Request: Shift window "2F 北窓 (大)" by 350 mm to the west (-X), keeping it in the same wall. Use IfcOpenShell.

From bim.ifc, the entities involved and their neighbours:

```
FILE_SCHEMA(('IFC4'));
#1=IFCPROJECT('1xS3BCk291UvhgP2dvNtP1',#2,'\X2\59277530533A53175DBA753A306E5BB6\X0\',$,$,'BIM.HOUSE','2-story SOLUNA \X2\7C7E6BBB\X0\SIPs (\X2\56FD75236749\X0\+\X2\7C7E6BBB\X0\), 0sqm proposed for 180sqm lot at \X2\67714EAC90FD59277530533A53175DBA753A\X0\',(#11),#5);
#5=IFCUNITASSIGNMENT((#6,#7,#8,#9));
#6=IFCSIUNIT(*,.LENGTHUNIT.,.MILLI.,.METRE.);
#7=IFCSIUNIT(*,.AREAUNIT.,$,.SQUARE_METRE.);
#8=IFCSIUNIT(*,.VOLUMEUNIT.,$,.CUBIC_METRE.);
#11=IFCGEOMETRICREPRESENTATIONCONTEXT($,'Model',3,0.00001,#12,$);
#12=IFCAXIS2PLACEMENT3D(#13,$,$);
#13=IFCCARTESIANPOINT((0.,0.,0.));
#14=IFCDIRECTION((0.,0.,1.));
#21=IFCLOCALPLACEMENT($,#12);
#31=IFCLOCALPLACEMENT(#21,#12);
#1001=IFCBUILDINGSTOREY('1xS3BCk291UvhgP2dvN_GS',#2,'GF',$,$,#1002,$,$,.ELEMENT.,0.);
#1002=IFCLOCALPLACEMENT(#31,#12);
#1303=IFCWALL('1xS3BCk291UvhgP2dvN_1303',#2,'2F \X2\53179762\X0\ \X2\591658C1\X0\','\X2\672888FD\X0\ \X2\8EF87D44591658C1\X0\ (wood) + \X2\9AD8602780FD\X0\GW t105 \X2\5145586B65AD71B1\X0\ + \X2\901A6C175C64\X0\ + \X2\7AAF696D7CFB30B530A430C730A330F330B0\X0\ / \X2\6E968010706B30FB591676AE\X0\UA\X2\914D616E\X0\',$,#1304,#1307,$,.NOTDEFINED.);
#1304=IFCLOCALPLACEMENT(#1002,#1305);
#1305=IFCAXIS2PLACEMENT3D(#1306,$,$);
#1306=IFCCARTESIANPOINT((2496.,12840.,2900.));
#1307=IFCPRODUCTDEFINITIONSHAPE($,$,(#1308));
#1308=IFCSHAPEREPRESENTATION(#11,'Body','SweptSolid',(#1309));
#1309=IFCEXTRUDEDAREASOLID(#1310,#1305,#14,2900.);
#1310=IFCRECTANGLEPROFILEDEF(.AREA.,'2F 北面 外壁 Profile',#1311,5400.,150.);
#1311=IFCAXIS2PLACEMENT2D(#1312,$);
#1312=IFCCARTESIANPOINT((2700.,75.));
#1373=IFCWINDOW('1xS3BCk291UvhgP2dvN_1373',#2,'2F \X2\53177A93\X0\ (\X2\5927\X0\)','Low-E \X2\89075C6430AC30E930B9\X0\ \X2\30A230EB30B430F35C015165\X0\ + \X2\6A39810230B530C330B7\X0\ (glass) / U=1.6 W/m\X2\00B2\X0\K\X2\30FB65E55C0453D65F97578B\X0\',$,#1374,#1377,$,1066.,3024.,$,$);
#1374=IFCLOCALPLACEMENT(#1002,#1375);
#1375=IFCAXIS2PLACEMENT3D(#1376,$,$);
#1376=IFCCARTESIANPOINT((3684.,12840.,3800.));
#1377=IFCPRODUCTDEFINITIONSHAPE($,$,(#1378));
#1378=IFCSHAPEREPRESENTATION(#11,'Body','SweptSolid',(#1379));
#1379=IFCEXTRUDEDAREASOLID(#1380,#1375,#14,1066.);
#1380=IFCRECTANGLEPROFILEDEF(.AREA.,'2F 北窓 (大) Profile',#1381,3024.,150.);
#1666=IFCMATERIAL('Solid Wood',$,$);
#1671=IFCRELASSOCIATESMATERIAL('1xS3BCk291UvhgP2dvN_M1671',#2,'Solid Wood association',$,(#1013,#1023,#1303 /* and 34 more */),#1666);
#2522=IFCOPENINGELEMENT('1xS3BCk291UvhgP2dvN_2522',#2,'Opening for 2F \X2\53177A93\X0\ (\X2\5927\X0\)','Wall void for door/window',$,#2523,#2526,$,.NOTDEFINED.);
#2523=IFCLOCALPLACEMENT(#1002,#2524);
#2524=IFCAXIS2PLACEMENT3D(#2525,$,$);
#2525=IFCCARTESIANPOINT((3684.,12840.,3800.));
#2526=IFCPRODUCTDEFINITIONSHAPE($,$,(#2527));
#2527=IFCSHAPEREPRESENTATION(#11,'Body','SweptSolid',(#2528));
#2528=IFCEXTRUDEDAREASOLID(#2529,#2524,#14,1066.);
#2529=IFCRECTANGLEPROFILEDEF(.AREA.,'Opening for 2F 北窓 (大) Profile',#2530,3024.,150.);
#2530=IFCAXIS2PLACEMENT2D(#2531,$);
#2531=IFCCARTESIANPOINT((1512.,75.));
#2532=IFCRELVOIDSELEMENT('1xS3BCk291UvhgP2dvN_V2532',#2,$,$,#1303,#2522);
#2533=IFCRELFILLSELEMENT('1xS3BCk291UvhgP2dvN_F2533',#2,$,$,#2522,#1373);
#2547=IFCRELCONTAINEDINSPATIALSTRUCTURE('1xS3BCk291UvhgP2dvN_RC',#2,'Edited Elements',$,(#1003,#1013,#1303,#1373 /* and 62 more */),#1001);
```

```python
import ifcopenshell
import ifcopenshell.api.geometry
import ifcopenshell.util.placement
import ifcopenshell.util.unit

model = ifcopenshell.open("bim.ifc")
unit_scale = ifcopenshell.util.unit.calculate_unit_scale(model)

window = model.by_guid("1xS3BCk291UvhgP2dvN_1373")
opening = window.FillsVoids[0].RelatingOpeningElement
wall = opening.VoidsElements[0].RelatingBuildingElement

wall_matrix = ifcopenshell.util.placement.get_local_placement(wall.ObjectPlacement)
shift = wall_matrix[:3, 0] * -0.35 / unit_scale
before = ifcopenshell.util.placement.get_local_placement(window.ObjectPlacement)[:3, 3].copy()

# The window is not placed relative to its opening, so move both.
for product in (opening, window):
    matrix = ifcopenshell.util.placement.get_local_placement(product.ObjectPlacement)
    matrix[:3, 3] += shift
    ifcopenshell.api.geometry.edit_object_placement(model, product=product, matrix=matrix, is_si=False)

after = ifcopenshell.util.placement.get_local_placement(window.ObjectPlacement)[:3, 3]
print("window moved by", (after - before).round(3) + 0.0)

model.write("bim_updated.ifc")
```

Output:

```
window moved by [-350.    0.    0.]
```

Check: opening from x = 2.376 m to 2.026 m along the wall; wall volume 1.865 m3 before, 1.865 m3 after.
